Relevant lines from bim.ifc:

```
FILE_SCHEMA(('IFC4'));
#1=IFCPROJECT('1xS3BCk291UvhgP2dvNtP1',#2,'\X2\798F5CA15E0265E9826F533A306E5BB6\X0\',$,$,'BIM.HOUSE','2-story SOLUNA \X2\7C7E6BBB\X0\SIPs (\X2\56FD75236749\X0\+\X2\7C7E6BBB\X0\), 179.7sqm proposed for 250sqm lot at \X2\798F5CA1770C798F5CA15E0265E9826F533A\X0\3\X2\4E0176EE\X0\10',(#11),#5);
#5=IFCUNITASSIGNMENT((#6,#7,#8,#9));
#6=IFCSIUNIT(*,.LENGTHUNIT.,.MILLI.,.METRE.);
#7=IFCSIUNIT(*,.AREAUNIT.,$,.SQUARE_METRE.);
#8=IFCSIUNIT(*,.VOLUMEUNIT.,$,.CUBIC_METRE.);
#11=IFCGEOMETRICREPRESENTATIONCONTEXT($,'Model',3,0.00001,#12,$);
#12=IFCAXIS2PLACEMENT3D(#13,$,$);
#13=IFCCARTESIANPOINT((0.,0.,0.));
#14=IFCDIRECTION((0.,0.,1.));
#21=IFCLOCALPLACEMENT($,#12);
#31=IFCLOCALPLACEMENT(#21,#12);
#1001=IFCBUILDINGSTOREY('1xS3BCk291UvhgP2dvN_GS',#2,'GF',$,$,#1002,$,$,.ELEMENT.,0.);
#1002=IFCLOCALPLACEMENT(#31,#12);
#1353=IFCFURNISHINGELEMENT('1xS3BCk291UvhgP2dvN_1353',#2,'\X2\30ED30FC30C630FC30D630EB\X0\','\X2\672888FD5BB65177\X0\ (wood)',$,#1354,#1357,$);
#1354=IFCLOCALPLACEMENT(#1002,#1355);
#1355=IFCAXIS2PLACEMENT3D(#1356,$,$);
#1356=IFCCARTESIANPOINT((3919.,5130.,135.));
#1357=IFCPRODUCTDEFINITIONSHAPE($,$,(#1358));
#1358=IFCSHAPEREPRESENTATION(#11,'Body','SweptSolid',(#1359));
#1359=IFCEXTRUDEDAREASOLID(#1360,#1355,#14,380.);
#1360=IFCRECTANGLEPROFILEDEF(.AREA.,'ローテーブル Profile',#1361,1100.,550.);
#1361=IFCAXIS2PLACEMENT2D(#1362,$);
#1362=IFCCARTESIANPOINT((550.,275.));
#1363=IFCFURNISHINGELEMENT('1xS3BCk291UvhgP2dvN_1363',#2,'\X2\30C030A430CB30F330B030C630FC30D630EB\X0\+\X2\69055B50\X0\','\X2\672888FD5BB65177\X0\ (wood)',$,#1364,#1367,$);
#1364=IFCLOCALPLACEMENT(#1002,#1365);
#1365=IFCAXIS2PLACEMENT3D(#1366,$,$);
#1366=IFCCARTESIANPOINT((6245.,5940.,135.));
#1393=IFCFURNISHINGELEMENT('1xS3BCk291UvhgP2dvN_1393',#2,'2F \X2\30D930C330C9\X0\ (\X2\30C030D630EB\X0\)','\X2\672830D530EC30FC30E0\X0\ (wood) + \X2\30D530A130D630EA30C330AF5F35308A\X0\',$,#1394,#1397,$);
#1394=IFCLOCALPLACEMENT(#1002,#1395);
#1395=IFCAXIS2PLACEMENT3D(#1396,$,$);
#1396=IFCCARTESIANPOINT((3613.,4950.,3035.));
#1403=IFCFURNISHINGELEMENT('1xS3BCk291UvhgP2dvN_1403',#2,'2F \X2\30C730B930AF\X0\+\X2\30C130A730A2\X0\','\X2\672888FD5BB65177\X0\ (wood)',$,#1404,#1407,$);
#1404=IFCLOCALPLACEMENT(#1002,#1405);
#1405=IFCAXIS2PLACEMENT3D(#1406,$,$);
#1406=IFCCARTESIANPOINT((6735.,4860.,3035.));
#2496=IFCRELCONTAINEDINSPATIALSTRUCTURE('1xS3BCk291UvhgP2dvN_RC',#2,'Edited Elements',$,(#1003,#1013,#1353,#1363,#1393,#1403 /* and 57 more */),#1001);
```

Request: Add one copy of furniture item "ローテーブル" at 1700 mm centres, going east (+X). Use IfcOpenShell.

```python
import numpy as np
import ifcopenshell
import ifcopenshell.api.geometry
import ifcopenshell.api.root
import ifcopenshell.util.element
import ifcopenshell.util.placement

model = ifcopenshell.open("bim.ifc")


def reuse_history(source, copy):
    """copy_class also copies each property set's owner history, people and application; keep the originals."""
    for rel in copy.IsDefinedBy:
        if rel.is_a("IfcRelDefinesByProperties") and (history := rel.RelatingPropertyDefinition.OwnerHistory):
            rel.RelatingPropertyDefinition.OwnerHistory = source.OwnerHistory
            ifcopenshell.util.element.remove_deep2(model, history)


source = model.by_guid("1xS3BCk291UvhgP2dvN_1353")
base = ifcopenshell.util.placement.get_local_placement(source.ObjectPlacement)
step = np.array([1.0, 0.0, 0.0]) * 1700.0

for i in range(1, 2):
    copy = ifcopenshell.api.root.copy_class(model, product=source)
    copy.Representation = ifcopenshell.util.element.copy_deep(
        model, source.Representation, exclude=["IfcGeometricRepresentationContext", "IfcRepresentationMap"]
    )
    reuse_history(source, copy)
    matrix = base.copy()
    matrix[:3, 3] += i * step
    print("added at", matrix[:3, 3].round(3) + 0.0)
    ifcopenshell.api.geometry.edit_object_placement(model, product=copy, matrix=matrix, is_si=False)

model.write("bim-out.ifc")
```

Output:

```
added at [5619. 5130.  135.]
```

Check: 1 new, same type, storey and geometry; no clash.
